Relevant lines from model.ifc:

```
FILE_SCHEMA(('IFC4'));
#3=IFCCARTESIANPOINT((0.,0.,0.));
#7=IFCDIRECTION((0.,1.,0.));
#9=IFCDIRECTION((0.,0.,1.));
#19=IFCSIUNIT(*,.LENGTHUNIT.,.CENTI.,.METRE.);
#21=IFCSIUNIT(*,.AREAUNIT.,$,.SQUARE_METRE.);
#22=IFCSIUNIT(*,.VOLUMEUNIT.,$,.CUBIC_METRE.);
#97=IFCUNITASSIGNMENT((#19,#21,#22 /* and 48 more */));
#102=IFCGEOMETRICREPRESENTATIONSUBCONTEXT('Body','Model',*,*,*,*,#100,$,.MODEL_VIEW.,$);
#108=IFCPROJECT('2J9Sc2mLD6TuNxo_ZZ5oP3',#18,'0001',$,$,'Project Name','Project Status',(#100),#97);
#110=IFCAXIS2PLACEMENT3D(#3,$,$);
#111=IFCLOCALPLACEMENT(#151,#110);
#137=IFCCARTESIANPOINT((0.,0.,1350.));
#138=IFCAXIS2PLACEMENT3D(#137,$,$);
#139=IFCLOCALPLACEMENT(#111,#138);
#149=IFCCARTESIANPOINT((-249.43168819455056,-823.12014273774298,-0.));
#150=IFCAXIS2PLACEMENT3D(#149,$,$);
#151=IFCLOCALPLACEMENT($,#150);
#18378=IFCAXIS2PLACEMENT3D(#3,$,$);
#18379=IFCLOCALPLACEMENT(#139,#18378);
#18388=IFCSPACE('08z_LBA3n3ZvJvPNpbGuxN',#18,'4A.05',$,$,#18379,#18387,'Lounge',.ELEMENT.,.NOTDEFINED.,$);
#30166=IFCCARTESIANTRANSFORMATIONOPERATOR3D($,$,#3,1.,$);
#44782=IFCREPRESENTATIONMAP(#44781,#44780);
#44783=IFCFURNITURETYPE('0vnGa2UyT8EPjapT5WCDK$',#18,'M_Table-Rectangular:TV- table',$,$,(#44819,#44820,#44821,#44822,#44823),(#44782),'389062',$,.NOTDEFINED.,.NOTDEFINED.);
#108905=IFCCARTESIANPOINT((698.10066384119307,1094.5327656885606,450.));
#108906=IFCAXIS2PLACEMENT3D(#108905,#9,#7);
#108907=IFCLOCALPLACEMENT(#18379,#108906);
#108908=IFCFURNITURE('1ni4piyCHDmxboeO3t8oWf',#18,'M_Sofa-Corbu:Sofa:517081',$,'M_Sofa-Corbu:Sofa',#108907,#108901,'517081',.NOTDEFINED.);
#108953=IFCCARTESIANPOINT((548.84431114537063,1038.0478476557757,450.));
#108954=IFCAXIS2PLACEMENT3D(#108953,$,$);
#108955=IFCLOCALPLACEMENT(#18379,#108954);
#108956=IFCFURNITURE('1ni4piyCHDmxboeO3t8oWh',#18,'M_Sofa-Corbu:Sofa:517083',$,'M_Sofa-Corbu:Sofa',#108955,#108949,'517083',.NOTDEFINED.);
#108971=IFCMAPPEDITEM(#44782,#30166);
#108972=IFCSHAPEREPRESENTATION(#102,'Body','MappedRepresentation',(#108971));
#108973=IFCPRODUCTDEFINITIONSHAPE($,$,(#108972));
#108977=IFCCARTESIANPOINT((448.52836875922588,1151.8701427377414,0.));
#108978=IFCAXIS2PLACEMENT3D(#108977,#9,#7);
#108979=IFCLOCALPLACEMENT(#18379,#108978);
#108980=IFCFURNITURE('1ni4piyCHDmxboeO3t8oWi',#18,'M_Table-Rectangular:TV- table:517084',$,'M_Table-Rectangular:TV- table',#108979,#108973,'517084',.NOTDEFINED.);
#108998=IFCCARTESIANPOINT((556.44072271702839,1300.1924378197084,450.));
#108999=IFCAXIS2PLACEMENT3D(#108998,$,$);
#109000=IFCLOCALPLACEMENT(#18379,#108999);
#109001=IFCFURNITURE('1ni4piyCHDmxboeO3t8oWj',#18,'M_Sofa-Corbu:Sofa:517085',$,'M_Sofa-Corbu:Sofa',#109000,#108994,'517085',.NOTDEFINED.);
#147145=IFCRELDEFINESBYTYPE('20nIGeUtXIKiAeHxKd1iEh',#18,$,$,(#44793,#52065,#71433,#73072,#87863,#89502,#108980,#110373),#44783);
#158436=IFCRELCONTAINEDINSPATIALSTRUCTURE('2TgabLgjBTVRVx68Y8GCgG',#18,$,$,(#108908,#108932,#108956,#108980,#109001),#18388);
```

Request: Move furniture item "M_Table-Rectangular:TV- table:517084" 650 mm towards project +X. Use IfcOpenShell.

```python
import ifcopenshell
import ifcopenshell.api.geometry
import ifcopenshell.util.placement
import ifcopenshell.util.unit

model = ifcopenshell.open("model.ifc")
unit_scale = ifcopenshell.util.unit.calculate_unit_scale(model)

item = model.by_id(108980)
matrix = ifcopenshell.util.placement.get_local_placement(item.ObjectPlacement)
matrix[0, 3] += 0.65 / unit_scale
ifcopenshell.api.geometry.edit_object_placement(model, product=item, matrix=matrix, is_si=False)

print(ifcopenshell.util.placement.get_local_placement(item.ObjectPlacement).round(3) + 0.0)

model.write("model_edited.ifc")
```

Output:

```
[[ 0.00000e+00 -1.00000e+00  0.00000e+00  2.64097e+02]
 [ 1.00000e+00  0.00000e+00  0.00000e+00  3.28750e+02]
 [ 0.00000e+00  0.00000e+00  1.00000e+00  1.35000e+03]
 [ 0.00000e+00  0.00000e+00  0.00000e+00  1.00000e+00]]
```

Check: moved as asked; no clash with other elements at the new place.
